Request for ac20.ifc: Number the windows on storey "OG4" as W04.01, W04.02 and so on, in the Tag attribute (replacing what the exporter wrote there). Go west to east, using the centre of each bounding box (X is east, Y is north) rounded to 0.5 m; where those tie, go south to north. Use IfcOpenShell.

First a look at what the model holds.

```python
import ifcopenshell
import ifcopenshell.util.element
import ifcopenshell.util.placement

model = ifcopenshell.open("ac20.ifc")
print(model.schema)
storey = next(s for s in model.by_type("IfcBuildingStorey") if s.Name == "OG4")
windows = [e for e in ifcopenshell.util.element.get_decomposition(storey) if e.is_a("IfcWindow")]
for e in sorted(windows, key=lambda e: e.id()):
    origin = ifcopenshell.util.placement.get_local_placement(e.ObjectPlacement)[:3, 3]
    print(e.id(), e.Tag, e.Name, origin.round(2) + 0.0, sep=" | ")
```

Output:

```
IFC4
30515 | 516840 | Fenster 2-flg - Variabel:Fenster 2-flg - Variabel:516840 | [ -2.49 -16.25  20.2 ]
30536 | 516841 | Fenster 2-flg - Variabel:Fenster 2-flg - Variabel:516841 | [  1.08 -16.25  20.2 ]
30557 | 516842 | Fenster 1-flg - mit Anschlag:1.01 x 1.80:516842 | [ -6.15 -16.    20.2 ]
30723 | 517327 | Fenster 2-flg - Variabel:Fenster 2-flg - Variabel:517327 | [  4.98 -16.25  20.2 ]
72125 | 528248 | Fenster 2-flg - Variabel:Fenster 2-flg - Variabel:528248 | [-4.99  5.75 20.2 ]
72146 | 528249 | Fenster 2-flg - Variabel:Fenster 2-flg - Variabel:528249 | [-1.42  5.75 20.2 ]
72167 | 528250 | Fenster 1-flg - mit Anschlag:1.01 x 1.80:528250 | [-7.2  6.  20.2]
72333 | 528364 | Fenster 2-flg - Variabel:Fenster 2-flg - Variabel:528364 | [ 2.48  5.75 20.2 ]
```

```python
import ifcopenshell
import ifcopenshell.geom
import ifcopenshell.util.element
import ifcopenshell.util.shape

model = ifcopenshell.open("ac20.ifc")
settings = ifcopenshell.geom.settings()
settings.set("use-world-coords", True)


def centre(element):
    shape = ifcopenshell.geom.create_shape(settings, element)
    return ifcopenshell.util.shape.get_bbox_centroid(shape.geometry)


storey = next(s for s in model.by_type("IfcBuildingStorey") if s.Name == "OG4")
windows = [e for e in ifcopenshell.util.element.get_decomposition(storey) if e.is_a("IfcWindow")]

# Insertion points can sit at a corner or the storey origin, so sort by the geometry (in metres).
centres = {e: centre(e) for e in windows}
windows.sort(key=lambda e: (round(centres[e][0] / 0.5), centres[e][1]))

for i, e in enumerate(windows, start=1):
    number = f"W04.{i:02d}"
    e.Tag = number
    print(e.id(), number)

model.write("ac20_updated.ifc")
```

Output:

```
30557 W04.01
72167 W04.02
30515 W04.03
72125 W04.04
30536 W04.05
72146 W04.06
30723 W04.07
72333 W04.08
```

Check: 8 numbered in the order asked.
